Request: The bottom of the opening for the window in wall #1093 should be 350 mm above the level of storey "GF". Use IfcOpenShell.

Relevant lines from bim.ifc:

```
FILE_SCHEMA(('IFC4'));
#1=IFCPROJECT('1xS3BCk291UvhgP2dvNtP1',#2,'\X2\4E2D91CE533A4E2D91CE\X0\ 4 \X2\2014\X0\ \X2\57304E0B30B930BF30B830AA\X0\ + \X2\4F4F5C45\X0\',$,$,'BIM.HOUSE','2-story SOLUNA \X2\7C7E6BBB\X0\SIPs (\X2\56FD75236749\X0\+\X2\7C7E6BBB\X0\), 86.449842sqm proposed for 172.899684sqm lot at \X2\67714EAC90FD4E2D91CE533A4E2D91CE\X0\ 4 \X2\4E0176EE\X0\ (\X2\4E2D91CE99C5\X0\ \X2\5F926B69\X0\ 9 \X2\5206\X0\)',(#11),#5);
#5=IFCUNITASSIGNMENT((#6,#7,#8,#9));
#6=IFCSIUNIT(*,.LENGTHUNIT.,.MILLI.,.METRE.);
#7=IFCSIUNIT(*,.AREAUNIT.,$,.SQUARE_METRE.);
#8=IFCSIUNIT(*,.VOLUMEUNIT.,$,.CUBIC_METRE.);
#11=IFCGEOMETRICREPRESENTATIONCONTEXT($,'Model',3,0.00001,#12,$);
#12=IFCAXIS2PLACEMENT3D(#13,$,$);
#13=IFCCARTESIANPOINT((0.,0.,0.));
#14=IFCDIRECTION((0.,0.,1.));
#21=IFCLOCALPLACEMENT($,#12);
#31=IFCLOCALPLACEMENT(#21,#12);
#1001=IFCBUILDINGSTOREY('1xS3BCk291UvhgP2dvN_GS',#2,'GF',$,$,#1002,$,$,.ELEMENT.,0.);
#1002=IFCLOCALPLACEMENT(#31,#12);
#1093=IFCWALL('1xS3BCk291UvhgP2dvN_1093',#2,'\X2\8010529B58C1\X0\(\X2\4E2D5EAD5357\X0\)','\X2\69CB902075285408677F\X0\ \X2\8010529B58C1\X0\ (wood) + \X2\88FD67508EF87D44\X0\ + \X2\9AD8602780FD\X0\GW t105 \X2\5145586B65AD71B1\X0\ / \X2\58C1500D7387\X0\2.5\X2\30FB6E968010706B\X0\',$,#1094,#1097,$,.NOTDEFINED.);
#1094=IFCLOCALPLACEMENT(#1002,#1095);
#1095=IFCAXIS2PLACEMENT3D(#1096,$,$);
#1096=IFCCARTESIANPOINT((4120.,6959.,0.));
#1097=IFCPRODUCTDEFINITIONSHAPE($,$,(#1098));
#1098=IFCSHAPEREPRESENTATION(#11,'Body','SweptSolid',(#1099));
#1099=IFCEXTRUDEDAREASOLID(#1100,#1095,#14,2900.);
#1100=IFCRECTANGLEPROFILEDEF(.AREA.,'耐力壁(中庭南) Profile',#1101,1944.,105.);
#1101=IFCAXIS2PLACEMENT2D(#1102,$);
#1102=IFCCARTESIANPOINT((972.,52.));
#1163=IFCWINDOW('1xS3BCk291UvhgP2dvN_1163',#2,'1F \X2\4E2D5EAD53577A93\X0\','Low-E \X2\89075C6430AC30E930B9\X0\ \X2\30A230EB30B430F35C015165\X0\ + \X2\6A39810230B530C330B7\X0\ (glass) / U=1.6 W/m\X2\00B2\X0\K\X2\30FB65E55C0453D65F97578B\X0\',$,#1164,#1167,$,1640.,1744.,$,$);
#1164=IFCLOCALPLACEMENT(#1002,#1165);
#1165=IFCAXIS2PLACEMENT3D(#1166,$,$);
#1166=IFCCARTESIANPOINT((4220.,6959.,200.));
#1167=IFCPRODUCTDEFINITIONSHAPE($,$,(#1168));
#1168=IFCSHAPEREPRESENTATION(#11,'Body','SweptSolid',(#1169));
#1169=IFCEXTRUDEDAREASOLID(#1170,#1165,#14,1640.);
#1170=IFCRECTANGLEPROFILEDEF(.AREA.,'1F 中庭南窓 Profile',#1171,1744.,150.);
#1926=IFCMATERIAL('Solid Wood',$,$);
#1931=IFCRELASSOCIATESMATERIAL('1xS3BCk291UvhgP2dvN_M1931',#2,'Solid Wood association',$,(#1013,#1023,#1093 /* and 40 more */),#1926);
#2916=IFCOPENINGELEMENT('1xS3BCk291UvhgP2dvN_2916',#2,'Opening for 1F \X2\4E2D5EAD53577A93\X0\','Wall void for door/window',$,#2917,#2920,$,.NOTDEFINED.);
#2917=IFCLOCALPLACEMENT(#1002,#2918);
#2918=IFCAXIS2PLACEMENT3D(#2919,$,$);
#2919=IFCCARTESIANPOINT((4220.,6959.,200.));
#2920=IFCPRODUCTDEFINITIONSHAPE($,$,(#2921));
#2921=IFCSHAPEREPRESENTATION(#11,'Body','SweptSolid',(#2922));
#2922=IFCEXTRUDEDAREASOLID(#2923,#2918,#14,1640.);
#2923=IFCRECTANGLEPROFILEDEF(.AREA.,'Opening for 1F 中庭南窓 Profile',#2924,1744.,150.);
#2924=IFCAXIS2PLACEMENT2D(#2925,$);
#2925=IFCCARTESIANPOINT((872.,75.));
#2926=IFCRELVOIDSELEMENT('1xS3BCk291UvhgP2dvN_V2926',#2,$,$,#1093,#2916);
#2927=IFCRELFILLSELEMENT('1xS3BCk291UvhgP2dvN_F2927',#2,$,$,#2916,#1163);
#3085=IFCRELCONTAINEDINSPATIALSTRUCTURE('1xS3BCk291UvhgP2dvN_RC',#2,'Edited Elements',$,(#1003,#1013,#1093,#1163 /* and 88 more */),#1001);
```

```python
import numpy as np
import ifcopenshell
import ifcopenshell.api.geometry
import ifcopenshell.geom
import ifcopenshell.util.element
import ifcopenshell.util.placement
import ifcopenshell.util.shape
import ifcopenshell.util.unit

model = ifcopenshell.open("bim.ifc")
unit_scale = ifcopenshell.util.unit.calculate_unit_scale(model)

window = model.by_id(1163)
opening = window.FillsVoids[0].RelatingOpeningElement
storey = ifcopenshell.util.element.get_container(window, ifc_class="IfcBuildingStorey")
level = ifcopenshell.util.placement.get_local_placement(storey.ObjectPlacement)[2, 3]

# The opening's origin need not be at the sill, so measure its lowest point.
shape = ifcopenshell.geom.create_shape(ifcopenshell.geom.settings(), opening)
bottom = ifcopenshell.util.shape.get_shape_bottom_elevation(shape, shape.geometry) / unit_scale
dz = level + 0.35 / unit_scale - bottom

shift = np.array([0.0, 0.0, dz])
# The window is not placed relative to its opening, so move both.
for product in (opening, window):
    matrix = ifcopenshell.util.placement.get_local_placement(product.ObjectPlacement)
    matrix[:3, 3] += shift
    ifcopenshell.api.geometry.edit_object_placement(model, product=product, matrix=matrix, is_si=False)

print(f"moved by {dz * unit_scale:+.3f} m")

model.write("bim_v2.ifc")
```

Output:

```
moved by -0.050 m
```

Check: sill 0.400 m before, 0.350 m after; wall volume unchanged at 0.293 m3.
